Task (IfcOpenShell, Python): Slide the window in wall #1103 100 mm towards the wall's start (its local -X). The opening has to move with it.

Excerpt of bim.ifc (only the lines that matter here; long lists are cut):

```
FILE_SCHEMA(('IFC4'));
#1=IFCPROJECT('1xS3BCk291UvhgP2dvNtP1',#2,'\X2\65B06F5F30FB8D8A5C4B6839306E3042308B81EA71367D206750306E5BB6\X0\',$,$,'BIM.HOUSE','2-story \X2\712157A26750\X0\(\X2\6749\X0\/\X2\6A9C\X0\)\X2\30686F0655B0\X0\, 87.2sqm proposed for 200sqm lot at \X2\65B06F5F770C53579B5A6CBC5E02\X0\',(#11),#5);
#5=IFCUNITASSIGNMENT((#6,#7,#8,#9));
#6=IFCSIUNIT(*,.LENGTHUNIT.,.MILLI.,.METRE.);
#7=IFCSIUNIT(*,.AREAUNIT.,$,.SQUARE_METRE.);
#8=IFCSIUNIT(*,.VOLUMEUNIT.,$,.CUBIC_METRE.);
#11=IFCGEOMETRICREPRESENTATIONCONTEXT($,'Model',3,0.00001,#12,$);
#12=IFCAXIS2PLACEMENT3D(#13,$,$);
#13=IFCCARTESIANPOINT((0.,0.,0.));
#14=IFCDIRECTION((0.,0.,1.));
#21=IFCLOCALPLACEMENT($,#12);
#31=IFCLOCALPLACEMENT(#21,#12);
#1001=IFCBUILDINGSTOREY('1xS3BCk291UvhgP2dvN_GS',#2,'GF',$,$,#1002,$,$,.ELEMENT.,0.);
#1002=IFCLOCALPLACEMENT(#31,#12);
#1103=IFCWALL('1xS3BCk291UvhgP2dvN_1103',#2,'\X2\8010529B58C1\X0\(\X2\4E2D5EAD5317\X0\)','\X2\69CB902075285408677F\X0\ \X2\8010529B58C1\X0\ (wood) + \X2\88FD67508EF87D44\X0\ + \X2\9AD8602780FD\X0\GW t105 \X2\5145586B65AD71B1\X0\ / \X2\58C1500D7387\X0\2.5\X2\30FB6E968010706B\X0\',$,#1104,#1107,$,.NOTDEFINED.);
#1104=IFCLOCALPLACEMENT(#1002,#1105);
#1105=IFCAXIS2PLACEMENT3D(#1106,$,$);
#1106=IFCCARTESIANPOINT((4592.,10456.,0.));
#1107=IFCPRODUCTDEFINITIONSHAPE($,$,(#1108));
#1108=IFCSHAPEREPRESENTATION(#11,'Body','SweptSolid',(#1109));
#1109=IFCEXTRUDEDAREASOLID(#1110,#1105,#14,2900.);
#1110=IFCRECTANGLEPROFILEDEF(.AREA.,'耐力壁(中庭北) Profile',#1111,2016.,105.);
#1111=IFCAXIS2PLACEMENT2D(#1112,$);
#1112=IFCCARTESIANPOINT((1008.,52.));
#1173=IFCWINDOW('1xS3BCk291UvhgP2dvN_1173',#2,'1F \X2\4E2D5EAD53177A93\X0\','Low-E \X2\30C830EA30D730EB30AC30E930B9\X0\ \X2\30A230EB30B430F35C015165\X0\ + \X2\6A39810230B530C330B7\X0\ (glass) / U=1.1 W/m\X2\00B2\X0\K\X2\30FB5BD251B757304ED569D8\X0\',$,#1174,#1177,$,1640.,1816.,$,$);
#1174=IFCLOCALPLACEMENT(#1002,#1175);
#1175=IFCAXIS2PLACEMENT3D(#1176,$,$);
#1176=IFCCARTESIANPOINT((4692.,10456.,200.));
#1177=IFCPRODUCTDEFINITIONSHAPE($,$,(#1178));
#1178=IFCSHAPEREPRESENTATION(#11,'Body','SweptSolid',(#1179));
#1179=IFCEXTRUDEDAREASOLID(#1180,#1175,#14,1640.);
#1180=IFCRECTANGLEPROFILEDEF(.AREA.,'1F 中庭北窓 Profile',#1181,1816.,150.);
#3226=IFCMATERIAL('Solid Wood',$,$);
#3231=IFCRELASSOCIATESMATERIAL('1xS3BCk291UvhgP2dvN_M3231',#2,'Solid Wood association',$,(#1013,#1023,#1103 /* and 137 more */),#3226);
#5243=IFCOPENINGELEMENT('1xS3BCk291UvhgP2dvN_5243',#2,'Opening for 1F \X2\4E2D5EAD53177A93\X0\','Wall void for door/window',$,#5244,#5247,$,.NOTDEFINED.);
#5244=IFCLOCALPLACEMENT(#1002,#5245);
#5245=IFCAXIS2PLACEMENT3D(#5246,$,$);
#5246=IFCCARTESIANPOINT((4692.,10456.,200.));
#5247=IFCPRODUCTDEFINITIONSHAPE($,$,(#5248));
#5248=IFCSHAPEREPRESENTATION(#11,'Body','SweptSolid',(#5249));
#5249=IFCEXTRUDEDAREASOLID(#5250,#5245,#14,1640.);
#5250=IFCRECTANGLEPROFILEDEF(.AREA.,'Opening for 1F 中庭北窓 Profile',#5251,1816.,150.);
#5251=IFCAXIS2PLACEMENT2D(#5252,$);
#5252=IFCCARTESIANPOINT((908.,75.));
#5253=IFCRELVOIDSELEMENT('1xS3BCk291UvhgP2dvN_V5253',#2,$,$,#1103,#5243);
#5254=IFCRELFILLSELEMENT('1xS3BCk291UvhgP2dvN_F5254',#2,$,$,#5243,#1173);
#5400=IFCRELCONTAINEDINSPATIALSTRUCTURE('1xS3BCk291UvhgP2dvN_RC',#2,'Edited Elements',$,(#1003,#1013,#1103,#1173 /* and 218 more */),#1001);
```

```python
import ifcopenshell
import ifcopenshell.api.geometry
import ifcopenshell.util.placement
import ifcopenshell.util.unit

model = ifcopenshell.open("bim.ifc")
unit_scale = ifcopenshell.util.unit.calculate_unit_scale(model)

window = model.by_id(1173)
opening = window.FillsVoids[0].RelatingOpeningElement
wall = opening.VoidsElements[0].RelatingBuildingElement

wall_matrix = ifcopenshell.util.placement.get_local_placement(wall.ObjectPlacement)
shift = wall_matrix[:3, 0] * -0.1 / unit_scale
before = ifcopenshell.util.placement.get_local_placement(window.ObjectPlacement)[:3, 3].copy()

# The window is not placed relative to its opening, so move both.
for product in (opening, window):
    matrix = ifcopenshell.util.placement.get_local_placement(product.ObjectPlacement)
    matrix[:3, 3] += shift
    ifcopenshell.api.geometry.edit_object_placement(model, product=product, matrix=matrix, is_si=False)

after = ifcopenshell.util.placement.get_local_placement(window.ObjectPlacement)[:3, 3]
print("window moved by", (after - before).round(3) + 0.0)

model.write("bim_edited.ifc")
```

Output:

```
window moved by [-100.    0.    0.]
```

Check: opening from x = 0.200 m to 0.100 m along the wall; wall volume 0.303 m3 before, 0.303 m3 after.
